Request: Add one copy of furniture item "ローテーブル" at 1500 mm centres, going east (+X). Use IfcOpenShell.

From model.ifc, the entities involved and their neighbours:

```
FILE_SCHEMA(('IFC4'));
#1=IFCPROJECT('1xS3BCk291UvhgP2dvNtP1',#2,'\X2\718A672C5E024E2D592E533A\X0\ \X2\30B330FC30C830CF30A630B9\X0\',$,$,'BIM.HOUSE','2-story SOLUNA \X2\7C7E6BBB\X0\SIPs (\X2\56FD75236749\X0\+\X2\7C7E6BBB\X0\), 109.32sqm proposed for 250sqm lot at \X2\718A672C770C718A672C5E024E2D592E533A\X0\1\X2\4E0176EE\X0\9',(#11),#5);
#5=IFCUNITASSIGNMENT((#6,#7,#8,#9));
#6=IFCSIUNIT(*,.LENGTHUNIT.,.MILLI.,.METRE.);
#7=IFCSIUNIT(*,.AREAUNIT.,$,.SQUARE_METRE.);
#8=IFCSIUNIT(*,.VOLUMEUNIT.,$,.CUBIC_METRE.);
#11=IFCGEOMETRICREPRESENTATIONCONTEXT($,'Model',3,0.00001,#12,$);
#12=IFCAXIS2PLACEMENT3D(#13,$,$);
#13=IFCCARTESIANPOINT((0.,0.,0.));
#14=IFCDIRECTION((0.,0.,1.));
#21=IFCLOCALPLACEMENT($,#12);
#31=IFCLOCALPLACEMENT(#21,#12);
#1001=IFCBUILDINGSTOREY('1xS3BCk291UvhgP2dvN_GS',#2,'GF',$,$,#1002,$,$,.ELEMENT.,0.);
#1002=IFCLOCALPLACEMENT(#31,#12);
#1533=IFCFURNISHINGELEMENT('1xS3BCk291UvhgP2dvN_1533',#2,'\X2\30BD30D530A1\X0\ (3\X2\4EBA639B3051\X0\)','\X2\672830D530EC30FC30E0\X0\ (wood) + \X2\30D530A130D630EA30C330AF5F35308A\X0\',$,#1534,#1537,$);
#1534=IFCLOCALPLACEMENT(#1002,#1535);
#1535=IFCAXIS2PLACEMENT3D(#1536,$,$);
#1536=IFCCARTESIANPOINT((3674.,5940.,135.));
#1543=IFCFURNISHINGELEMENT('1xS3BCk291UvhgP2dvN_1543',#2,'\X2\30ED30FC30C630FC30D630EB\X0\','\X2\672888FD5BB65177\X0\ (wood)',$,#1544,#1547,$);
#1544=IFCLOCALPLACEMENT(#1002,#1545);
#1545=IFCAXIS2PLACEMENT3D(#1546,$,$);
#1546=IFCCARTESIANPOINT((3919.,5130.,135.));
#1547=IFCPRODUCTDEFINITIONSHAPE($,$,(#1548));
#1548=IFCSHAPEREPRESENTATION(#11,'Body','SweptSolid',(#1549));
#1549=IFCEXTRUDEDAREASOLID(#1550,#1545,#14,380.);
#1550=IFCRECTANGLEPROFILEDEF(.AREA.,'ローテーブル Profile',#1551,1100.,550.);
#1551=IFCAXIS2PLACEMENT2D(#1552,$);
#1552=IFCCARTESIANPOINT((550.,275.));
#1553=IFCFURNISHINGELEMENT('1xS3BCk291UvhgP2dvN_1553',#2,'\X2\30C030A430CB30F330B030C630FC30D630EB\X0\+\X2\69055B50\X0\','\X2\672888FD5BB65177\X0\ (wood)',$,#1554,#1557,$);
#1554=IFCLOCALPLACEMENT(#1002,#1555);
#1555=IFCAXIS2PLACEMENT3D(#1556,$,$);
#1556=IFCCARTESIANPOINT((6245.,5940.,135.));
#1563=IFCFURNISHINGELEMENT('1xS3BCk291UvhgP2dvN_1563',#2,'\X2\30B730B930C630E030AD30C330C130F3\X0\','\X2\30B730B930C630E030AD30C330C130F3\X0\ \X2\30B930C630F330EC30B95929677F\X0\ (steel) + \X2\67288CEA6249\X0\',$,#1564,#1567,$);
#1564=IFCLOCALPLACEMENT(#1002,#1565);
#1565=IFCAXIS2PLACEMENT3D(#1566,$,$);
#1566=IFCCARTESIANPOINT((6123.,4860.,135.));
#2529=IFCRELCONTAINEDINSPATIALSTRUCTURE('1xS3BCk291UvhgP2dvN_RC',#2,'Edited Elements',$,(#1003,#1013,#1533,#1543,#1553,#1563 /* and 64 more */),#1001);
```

```python
import numpy as np
import ifcopenshell
import ifcopenshell.api.geometry
import ifcopenshell.api.root
import ifcopenshell.util.element
import ifcopenshell.util.placement

model = ifcopenshell.open("model.ifc")


def reuse_history(source, copy):
    """copy_class also copies each property set's owner history, people and application; keep the originals."""
    for rel in copy.IsDefinedBy:
        if rel.is_a("IfcRelDefinesByProperties") and (history := rel.RelatingPropertyDefinition.OwnerHistory):
            rel.RelatingPropertyDefinition.OwnerHistory = source.OwnerHistory
            ifcopenshell.util.element.remove_deep2(model, history)


source = model.by_id(1543)
base = ifcopenshell.util.placement.get_local_placement(source.ObjectPlacement)
step = np.array([1.0, 0.0, 0.0]) * 1500.0

for i in range(1, 2):
    copy = ifcopenshell.api.root.copy_class(model, product=source)
    copy.Representation = ifcopenshell.util.element.copy_deep(
        model, source.Representation, exclude=["IfcGeometricRepresentationContext", "IfcRepresentationMap"]
    )
    reuse_history(source, copy)
    matrix = base.copy()
    matrix[:3, 3] += i * step
    print("added at", matrix[:3, 3].round(3) + 0.0)
    ifcopenshell.api.geometry.edit_object_placement(model, product=copy, matrix=matrix, is_si=False)

model.write("model_v2.ifc")
```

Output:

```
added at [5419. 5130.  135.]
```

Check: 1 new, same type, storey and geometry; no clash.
